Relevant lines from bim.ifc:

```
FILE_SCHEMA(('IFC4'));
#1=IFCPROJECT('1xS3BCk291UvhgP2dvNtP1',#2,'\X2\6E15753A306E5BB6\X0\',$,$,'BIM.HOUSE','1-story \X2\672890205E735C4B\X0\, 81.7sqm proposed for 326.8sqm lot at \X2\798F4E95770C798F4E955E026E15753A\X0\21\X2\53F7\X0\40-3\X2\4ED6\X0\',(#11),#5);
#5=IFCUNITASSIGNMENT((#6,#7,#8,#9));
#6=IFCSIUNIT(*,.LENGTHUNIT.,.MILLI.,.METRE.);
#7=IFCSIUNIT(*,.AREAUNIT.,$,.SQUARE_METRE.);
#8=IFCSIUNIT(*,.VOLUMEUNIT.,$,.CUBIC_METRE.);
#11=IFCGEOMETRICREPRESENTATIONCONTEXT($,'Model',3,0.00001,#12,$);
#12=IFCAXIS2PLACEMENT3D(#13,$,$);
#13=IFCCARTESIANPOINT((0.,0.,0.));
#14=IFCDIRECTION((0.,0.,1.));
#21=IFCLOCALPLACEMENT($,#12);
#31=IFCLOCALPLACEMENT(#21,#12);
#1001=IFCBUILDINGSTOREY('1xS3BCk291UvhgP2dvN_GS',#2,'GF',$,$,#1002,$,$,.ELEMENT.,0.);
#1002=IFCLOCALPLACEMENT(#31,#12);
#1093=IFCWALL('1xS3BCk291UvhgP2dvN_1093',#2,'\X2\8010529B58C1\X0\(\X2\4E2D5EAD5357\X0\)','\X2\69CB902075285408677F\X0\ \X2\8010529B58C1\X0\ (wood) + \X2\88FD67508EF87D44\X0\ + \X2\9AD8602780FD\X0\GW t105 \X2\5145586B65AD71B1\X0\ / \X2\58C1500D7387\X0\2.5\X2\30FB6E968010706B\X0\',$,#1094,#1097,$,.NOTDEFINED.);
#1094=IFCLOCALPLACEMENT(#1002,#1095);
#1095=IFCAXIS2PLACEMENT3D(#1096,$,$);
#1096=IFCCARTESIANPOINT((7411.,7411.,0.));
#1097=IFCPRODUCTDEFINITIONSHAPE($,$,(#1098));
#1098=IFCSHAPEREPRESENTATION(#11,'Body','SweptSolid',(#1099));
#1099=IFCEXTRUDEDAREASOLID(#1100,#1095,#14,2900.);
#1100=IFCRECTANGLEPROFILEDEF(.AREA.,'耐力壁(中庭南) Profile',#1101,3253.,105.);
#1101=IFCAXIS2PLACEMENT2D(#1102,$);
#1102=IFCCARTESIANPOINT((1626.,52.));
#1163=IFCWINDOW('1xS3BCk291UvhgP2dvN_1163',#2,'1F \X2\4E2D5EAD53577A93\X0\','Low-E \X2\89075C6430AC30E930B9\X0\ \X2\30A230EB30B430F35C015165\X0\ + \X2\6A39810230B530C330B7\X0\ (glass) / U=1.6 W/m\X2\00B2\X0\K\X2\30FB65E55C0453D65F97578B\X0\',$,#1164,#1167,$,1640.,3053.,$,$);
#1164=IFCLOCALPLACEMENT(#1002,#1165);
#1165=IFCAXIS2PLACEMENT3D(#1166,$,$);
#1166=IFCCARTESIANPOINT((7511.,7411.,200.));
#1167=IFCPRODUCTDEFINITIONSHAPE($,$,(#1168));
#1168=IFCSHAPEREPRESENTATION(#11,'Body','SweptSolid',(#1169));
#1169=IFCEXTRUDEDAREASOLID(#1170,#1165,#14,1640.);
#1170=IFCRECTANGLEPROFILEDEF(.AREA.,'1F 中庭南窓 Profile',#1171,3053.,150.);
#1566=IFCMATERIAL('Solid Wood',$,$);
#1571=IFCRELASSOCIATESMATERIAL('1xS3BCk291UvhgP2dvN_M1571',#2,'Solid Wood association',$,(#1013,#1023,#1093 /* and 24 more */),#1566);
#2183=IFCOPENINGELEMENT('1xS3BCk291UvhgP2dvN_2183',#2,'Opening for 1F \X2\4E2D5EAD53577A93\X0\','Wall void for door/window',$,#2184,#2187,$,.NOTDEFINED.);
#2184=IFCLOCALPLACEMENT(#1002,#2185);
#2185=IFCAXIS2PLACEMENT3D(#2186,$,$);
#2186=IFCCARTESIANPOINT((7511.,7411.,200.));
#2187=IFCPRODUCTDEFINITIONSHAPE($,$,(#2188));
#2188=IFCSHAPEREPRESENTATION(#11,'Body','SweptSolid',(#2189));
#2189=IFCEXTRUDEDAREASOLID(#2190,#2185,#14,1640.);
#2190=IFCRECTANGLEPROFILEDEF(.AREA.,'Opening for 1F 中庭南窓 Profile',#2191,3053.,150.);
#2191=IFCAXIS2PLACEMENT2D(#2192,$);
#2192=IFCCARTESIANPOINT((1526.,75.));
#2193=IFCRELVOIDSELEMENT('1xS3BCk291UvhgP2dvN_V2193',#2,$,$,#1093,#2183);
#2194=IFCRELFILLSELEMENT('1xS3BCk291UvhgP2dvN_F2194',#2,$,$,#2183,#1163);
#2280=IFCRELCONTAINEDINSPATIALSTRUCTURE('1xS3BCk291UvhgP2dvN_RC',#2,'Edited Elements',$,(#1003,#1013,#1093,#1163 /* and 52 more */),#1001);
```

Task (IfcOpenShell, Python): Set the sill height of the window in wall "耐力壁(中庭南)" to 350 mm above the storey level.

```python
import numpy as np
import ifcopenshell
import ifcopenshell.api.geometry
import ifcopenshell.geom
import ifcopenshell.util.element
import ifcopenshell.util.placement
import ifcopenshell.util.shape
import ifcopenshell.util.unit

model = ifcopenshell.open("bim.ifc")
unit_scale = ifcopenshell.util.unit.calculate_unit_scale(model)

window = model.by_guid("1xS3BCk291UvhgP2dvN_1163")
opening = window.FillsVoids[0].RelatingOpeningElement
storey = ifcopenshell.util.element.get_container(window, ifc_class="IfcBuildingStorey")
level = ifcopenshell.util.placement.get_local_placement(storey.ObjectPlacement)[2, 3]

# The opening's origin need not be at the sill, so measure its lowest point.
shape = ifcopenshell.geom.create_shape(ifcopenshell.geom.settings(), opening)
bottom = ifcopenshell.util.shape.get_shape_bottom_elevation(shape, shape.geometry) / unit_scale
dz = level + 0.35 / unit_scale - bottom

shift = np.array([0.0, 0.0, dz])
# The window is not placed relative to its opening, so move both.
for product in (opening, window):
    matrix = ifcopenshell.util.placement.get_local_placement(product.ObjectPlacement)
    matrix[:3, 3] += shift
    ifcopenshell.api.geometry.edit_object_placement(model, product=product, matrix=matrix, is_si=False)

print(f"moved by {dz * unit_scale:+.3f} m")

model.write("bim_rev.ifc")
```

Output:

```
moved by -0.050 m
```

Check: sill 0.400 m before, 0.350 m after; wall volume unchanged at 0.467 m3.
